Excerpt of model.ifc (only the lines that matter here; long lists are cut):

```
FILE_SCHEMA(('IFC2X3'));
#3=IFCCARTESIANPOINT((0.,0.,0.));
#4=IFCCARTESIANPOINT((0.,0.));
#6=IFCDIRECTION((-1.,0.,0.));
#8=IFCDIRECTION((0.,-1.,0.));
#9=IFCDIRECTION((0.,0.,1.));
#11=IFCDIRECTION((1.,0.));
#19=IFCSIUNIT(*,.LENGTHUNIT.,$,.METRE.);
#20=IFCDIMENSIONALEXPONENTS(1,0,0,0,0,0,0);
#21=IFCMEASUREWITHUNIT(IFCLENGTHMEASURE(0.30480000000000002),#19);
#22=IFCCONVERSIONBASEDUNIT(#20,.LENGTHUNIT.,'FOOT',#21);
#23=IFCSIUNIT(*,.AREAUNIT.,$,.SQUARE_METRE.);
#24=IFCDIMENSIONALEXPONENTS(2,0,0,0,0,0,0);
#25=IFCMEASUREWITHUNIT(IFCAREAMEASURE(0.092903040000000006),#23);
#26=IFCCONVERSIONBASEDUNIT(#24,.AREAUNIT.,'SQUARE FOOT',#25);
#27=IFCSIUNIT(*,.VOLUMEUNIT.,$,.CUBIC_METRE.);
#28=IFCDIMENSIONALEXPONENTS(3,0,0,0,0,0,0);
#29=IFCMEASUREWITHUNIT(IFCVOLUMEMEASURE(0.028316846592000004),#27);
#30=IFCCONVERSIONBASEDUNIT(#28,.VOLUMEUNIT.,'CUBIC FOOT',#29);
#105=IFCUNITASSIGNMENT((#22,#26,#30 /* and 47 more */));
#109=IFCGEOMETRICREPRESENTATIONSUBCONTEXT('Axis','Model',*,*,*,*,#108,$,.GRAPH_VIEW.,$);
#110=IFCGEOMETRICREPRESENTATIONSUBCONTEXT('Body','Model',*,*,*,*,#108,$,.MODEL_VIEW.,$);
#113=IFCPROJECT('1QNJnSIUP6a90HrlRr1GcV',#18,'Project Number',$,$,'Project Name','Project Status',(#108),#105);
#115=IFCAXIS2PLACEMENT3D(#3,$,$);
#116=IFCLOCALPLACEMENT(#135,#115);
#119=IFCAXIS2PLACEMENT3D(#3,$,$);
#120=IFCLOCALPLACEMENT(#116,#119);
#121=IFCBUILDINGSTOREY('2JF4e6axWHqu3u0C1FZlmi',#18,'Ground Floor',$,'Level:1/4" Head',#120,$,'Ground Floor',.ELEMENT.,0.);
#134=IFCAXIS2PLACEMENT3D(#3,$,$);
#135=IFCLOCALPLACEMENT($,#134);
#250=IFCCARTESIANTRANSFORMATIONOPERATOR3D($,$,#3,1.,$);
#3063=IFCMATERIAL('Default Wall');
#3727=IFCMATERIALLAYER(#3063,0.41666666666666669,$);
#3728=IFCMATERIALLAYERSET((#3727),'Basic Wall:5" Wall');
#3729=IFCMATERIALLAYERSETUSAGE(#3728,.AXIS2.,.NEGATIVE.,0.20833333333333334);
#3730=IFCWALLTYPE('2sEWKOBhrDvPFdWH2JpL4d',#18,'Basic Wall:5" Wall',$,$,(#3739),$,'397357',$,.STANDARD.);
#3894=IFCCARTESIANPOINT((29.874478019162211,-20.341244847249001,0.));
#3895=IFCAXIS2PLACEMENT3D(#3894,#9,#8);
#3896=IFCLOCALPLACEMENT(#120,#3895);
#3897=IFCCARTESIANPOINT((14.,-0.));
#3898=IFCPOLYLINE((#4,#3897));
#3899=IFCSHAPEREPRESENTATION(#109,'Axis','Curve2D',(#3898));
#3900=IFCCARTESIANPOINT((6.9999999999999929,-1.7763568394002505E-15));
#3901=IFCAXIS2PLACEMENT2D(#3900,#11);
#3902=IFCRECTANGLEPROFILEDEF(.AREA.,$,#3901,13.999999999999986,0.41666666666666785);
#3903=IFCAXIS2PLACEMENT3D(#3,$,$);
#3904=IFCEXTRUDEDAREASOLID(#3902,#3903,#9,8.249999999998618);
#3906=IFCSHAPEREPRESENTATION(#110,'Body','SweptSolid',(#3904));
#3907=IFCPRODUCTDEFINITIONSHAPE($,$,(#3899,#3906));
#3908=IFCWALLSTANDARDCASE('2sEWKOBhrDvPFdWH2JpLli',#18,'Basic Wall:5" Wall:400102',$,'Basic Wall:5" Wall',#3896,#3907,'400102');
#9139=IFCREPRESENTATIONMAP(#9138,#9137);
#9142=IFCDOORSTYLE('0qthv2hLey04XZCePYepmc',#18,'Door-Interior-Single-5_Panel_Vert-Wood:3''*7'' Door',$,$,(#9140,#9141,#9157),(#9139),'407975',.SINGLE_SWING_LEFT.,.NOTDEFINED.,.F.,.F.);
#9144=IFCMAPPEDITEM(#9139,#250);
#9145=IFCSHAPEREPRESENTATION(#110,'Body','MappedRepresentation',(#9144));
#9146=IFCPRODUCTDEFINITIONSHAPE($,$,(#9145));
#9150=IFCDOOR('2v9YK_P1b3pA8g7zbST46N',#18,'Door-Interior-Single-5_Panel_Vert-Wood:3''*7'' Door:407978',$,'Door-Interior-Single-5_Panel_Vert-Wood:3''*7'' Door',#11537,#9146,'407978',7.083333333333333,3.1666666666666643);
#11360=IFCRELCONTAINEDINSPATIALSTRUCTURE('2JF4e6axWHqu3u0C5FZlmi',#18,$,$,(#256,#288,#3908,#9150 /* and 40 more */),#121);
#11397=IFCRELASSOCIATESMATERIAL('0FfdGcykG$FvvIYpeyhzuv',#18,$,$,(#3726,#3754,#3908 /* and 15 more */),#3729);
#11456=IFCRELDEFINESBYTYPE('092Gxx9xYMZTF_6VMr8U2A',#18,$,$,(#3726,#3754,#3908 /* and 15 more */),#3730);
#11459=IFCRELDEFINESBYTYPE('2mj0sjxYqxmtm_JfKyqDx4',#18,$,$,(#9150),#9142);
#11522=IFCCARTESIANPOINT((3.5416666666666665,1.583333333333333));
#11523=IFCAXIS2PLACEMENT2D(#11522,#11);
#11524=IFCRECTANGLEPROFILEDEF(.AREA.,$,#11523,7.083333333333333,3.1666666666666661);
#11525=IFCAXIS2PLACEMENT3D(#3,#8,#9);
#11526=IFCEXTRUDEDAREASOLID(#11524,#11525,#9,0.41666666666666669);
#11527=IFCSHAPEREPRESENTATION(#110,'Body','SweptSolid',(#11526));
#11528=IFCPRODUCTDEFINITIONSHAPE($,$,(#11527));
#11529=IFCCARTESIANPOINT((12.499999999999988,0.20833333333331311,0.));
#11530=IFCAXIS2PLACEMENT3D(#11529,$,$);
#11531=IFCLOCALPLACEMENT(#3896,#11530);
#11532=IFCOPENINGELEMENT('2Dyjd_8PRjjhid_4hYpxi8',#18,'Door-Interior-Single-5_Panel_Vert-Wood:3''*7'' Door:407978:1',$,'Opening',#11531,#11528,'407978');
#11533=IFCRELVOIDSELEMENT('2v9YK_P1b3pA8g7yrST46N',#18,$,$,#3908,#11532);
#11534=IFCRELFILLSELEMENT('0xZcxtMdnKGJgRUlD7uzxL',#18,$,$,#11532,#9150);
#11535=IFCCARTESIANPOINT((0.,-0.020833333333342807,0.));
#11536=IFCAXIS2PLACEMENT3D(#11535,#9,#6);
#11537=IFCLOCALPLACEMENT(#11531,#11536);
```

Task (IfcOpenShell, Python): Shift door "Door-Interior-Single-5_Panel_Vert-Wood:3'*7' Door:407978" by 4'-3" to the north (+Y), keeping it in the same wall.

```python
import ifcopenshell
import ifcopenshell.api.geometry
import ifcopenshell.util.placement
import ifcopenshell.util.unit

model = ifcopenshell.open("model.ifc")
unit_scale = ifcopenshell.util.unit.calculate_unit_scale(model)

door = model.by_guid("2v9YK_P1b3pA8g7zbST46N")
opening = door.FillsVoids[0].RelatingOpeningElement
wall = opening.VoidsElements[0].RelatingBuildingElement

wall_matrix = ifcopenshell.util.placement.get_local_placement(wall.ObjectPlacement)
shift = wall_matrix[:3, 0] * -51 * 0.0254 / unit_scale
before = ifcopenshell.util.placement.get_local_placement(door.ObjectPlacement)[:3, 3].copy()

# The door is placed relative to its opening, so it follows when the opening moves.
matrix = ifcopenshell.util.placement.get_local_placement(opening.ObjectPlacement)
matrix[:3, 3] += shift
ifcopenshell.api.geometry.edit_object_placement(
    model, product=opening, matrix=matrix, is_si=False, should_transform_children=True
)

after = ifcopenshell.util.placement.get_local_placement(door.ObjectPlacement)[:3, 3]
print("door moved by", (after - before).round(3) + 0.0)

model.write("model_v2.ifc")
```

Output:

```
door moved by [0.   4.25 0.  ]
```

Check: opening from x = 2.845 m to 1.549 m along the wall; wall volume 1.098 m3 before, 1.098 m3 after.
